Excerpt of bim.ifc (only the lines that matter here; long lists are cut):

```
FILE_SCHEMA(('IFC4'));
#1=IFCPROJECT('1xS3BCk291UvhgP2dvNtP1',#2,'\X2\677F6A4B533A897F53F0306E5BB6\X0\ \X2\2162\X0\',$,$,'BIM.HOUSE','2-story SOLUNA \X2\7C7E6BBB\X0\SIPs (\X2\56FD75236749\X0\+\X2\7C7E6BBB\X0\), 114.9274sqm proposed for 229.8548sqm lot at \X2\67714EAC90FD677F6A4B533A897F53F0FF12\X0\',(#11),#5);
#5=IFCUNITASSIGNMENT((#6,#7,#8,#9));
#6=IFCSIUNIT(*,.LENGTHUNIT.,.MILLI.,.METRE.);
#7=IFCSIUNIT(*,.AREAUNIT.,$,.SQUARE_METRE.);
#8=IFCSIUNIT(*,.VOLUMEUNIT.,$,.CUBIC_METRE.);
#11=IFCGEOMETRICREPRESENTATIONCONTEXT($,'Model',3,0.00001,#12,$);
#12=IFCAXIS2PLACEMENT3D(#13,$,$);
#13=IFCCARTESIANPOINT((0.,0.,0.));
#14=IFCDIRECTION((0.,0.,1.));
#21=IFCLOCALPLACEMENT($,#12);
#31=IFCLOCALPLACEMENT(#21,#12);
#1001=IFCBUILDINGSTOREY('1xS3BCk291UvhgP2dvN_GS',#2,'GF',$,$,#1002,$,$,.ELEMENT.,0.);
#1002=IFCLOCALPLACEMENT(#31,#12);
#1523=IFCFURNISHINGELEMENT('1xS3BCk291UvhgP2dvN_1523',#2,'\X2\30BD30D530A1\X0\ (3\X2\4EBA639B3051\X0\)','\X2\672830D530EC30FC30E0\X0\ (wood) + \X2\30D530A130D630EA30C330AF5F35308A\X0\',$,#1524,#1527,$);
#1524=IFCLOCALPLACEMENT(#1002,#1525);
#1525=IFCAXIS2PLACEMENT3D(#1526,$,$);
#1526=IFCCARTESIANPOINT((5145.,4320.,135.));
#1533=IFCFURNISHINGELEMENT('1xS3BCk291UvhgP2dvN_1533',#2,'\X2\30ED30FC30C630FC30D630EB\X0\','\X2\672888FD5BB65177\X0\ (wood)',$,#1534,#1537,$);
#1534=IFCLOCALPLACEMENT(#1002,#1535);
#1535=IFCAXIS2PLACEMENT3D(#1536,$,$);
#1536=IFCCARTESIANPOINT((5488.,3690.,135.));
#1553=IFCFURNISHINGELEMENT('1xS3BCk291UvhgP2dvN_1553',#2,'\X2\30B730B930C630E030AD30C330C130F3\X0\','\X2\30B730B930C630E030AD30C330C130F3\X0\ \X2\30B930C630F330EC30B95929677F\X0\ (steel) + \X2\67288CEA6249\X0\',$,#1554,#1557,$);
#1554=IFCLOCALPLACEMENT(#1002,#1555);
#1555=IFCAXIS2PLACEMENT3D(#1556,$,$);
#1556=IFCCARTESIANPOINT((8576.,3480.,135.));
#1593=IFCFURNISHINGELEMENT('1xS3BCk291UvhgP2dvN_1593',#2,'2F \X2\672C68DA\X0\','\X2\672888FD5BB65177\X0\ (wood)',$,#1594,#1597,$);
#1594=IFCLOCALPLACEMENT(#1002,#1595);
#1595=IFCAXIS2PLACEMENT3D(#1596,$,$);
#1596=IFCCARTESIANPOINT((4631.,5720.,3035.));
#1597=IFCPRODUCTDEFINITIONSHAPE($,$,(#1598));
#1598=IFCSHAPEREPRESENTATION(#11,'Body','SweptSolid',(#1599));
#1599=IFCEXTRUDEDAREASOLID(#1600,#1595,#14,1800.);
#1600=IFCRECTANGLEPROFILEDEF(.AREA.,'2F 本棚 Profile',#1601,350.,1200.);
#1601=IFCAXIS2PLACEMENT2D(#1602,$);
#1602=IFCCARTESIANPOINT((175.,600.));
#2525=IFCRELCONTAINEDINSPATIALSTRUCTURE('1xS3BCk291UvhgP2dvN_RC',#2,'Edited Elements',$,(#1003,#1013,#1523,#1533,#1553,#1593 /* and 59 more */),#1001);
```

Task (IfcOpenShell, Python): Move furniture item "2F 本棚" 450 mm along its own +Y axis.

```python
import ifcopenshell
import ifcopenshell.api.geometry
import ifcopenshell.util.placement

model = ifcopenshell.open("bim.ifc")

item = model.by_id(1593)
matrix = ifcopenshell.util.placement.get_local_placement(item.ObjectPlacement)
matrix[:3, 3] += matrix[:3, 1] * 450.0
ifcopenshell.api.geometry.edit_object_placement(model, product=item, matrix=matrix, is_si=False)

print(ifcopenshell.util.placement.get_local_placement(item.ObjectPlacement).round(3) + 0.0)

model.write("bim_edited.ifc")
```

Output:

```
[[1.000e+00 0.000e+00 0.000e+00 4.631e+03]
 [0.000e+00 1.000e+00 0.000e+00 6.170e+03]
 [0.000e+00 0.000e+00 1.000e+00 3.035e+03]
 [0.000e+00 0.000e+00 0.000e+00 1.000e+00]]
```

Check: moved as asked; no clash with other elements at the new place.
